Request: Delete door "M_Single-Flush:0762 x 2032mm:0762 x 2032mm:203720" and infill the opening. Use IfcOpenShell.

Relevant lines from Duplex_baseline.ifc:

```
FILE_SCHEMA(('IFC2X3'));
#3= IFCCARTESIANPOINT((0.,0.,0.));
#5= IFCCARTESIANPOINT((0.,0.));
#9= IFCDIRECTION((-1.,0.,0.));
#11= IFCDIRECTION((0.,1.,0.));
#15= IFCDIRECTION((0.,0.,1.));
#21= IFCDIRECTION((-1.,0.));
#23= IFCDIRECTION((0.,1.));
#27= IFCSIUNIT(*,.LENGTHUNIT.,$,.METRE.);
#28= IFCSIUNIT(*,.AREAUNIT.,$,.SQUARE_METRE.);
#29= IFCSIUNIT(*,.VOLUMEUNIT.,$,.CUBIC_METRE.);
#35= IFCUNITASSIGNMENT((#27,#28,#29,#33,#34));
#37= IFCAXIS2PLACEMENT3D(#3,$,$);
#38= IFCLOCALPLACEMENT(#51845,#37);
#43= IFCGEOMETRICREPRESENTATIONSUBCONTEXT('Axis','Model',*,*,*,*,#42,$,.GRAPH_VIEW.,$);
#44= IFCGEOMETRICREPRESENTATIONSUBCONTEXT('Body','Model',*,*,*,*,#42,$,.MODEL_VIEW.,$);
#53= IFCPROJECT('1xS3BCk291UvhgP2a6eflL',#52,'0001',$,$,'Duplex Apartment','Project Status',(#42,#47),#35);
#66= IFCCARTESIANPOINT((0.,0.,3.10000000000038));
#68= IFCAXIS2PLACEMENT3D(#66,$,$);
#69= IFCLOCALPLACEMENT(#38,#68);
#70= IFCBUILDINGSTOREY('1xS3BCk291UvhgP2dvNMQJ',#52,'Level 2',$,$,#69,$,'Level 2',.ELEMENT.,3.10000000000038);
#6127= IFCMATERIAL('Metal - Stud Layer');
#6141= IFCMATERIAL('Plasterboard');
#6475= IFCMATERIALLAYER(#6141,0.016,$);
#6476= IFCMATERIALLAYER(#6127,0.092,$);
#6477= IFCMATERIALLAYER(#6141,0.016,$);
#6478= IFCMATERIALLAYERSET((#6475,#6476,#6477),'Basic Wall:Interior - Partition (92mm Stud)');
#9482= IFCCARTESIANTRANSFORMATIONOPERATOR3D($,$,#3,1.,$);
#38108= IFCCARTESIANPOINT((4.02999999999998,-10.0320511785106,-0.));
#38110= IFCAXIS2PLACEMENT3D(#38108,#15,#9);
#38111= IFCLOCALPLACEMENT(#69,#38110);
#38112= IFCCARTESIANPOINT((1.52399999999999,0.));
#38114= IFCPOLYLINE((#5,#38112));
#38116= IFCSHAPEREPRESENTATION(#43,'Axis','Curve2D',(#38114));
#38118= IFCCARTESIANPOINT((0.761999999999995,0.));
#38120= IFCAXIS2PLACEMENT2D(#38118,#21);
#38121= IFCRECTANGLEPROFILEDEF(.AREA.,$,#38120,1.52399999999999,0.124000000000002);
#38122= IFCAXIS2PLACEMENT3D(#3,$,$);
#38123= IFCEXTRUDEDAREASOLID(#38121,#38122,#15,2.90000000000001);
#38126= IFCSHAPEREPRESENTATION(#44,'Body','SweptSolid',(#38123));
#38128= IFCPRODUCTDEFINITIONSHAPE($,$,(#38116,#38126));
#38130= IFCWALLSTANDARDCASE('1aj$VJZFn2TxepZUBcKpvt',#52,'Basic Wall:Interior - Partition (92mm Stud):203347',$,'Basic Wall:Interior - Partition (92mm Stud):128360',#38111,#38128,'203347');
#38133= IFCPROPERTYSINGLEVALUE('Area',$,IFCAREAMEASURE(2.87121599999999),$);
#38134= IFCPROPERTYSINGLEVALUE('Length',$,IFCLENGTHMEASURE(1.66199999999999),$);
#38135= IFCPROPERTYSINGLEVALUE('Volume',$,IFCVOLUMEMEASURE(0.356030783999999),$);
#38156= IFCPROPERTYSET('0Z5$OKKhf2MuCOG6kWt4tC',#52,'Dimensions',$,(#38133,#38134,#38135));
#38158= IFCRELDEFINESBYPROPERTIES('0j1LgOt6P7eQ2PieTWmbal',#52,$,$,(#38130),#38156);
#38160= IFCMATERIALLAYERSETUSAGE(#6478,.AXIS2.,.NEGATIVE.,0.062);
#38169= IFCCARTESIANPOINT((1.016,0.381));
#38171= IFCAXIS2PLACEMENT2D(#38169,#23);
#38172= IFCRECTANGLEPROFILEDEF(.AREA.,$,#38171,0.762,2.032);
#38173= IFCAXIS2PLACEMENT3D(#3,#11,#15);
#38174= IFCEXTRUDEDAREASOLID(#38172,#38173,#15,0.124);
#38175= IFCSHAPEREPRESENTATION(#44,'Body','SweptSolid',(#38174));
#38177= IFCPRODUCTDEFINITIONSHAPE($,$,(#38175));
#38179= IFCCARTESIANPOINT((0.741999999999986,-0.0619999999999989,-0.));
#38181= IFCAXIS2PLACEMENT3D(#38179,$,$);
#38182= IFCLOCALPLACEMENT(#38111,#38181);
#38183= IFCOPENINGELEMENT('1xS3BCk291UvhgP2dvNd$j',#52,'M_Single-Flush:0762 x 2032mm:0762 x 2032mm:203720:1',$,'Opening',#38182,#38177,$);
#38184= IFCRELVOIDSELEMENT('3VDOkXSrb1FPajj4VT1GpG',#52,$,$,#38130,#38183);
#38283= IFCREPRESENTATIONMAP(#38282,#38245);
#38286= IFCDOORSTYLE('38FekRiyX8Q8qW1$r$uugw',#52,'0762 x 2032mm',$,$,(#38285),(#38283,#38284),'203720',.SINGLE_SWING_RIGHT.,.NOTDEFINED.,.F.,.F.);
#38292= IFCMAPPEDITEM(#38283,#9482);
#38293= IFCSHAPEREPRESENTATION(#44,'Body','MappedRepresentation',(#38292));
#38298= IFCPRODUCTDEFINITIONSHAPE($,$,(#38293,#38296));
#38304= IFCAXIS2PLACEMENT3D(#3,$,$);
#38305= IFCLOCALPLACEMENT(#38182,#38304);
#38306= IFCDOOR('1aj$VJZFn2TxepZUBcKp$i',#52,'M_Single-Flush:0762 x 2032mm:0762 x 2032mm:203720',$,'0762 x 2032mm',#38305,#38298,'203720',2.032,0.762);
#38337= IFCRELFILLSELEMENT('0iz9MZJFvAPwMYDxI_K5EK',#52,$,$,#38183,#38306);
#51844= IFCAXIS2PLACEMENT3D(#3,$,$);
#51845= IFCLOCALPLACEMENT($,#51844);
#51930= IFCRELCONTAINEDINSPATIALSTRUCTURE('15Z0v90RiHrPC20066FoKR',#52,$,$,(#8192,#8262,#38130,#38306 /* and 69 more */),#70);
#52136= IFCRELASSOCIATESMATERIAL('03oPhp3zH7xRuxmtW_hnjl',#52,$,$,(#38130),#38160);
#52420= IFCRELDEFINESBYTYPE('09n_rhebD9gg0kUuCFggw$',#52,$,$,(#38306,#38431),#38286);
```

```python
import ifcopenshell
import ifcopenshell.api.feature
import ifcopenshell.api.pset
import ifcopenshell.api.root
import ifcopenshell.geom
import ifcopenshell.util.element
import ifcopenshell.util.shape
import ifcopenshell.util.unit

model = ifcopenshell.open("Duplex_baseline.ifc")
area_scale = ifcopenshell.util.unit.calculate_unit_scale(model, "AREAUNIT")
volume_scale = ifcopenshell.util.unit.calculate_unit_scale(model, "VOLUMEUNIT")
settings = ifcopenshell.geom.settings()


def volume(element):
    """Net volume in cubic metres, openings subtracted."""
    shape = ifcopenshell.geom.create_shape(settings, element)
    return ifcopenshell.util.shape.get_volume(shape.geometry)


door = model.by_id(38306)
opening = door.FillsVoids[0].RelatingOpeningElement
wall = opening.VoidsElements[0].RelatingBuildingElement
before = volume(wall)

ifcopenshell.api.root.remove_product(model, product=door)
ifcopenshell.api.feature.remove_feature(model, feature=opening)

after = volume(wall)
thickness = 0.124  # wall thickness in metres

# Update the wall's stored quantities.
pset = model.by_id(ifcopenshell.util.element.get_pset(wall, "Dimensions", should_inherit=False)["id"])
ifcopenshell.api.pset.edit_pset(model, pset=pset, properties={
    "Area": model.create_entity("IfcAreaMeasure", after / thickness / area_scale),
    "Volume": model.create_entity("IfcVolumeMeasure", after / volume_scale),
})

print(f"wall volume {before:.3f} -> {after:.3f} m3")

model.write("Duplex_baseline_updated.ifc")
```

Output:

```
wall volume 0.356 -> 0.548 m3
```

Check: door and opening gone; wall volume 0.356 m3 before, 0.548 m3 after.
